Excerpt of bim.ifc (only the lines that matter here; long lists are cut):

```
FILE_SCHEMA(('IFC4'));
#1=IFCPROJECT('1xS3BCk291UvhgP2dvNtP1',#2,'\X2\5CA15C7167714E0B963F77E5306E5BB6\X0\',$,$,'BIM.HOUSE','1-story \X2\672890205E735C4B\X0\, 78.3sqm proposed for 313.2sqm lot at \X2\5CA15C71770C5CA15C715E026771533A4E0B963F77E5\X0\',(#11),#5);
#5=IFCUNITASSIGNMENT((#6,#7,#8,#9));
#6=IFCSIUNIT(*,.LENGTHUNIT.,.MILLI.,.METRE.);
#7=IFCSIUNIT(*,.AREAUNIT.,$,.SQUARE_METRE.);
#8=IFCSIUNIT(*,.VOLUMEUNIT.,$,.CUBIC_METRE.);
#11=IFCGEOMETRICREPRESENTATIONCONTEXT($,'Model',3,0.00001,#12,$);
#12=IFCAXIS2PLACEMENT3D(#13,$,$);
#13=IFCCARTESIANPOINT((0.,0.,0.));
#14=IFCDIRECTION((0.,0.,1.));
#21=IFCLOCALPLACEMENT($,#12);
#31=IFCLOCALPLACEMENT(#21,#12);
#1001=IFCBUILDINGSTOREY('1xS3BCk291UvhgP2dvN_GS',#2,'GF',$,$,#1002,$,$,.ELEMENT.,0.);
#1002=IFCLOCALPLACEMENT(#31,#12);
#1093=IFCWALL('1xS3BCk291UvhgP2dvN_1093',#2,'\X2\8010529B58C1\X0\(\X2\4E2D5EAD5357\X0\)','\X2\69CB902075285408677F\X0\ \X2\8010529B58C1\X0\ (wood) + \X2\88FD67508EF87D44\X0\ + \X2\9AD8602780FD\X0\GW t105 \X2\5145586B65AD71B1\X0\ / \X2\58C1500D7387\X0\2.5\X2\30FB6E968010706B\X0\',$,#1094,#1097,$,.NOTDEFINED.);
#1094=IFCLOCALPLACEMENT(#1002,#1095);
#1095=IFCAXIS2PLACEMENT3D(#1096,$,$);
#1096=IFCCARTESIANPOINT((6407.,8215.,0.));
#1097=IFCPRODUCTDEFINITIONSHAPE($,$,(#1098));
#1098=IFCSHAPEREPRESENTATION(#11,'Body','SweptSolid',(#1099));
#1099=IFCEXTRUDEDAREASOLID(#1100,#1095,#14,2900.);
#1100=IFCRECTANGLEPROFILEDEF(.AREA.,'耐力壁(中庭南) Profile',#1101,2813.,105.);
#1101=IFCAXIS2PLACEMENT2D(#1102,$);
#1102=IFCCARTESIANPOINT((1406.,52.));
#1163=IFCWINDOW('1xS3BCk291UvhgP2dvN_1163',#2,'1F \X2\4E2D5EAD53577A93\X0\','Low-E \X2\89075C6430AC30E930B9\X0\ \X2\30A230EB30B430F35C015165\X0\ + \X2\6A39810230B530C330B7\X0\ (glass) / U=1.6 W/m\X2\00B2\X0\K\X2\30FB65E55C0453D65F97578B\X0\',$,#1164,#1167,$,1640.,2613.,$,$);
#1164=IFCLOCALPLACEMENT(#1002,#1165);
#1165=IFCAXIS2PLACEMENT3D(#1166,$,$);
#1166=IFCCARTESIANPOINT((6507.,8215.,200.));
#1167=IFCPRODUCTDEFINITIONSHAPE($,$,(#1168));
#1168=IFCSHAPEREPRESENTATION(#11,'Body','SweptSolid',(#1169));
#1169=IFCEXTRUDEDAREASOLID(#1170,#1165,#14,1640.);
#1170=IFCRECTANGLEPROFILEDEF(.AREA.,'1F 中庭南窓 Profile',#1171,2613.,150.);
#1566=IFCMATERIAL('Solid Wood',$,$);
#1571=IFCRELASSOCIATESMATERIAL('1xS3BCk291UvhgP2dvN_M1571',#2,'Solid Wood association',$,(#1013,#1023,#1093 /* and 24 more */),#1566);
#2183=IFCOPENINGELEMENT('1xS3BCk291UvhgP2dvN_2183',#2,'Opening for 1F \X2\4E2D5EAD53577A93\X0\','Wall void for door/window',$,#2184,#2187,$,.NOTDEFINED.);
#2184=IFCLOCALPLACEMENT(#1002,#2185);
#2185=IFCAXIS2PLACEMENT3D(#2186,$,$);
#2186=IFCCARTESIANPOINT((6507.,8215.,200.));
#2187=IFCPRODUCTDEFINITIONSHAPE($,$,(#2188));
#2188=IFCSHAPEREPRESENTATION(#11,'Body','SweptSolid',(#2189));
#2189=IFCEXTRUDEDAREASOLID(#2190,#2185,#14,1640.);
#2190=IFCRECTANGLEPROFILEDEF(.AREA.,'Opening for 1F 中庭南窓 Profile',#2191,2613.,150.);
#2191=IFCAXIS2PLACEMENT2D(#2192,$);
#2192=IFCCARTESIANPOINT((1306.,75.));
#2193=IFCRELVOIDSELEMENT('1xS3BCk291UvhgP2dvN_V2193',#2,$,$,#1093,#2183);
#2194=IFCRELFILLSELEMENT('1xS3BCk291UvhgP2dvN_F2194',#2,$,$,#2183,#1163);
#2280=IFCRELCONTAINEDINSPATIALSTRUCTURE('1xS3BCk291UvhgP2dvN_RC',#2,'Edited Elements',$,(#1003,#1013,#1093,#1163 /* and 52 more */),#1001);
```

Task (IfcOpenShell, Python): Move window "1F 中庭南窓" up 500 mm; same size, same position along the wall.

```python
import numpy as np
import ifcopenshell
import ifcopenshell.api.geometry
import ifcopenshell.util.placement
import ifcopenshell.util.unit

model = ifcopenshell.open("bim.ifc")
unit_scale = ifcopenshell.util.unit.calculate_unit_scale(model)

window = model.by_guid("1xS3BCk291UvhgP2dvN_1163")
opening = window.FillsVoids[0].RelatingOpeningElement
dz = 0.5 / unit_scale

shift = np.array([0.0, 0.0, dz])
# The window is not placed relative to its opening, so move both.
for product in (opening, window):
    matrix = ifcopenshell.util.placement.get_local_placement(product.ObjectPlacement)
    matrix[:3, 3] += shift
    ifcopenshell.api.geometry.edit_object_placement(model, product=product, matrix=matrix, is_si=False)

print(f"moved by {dz * unit_scale:+.3f} m")

model.write("bim_rev.ifc")
```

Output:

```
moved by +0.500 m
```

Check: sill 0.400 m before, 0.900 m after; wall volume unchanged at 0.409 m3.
